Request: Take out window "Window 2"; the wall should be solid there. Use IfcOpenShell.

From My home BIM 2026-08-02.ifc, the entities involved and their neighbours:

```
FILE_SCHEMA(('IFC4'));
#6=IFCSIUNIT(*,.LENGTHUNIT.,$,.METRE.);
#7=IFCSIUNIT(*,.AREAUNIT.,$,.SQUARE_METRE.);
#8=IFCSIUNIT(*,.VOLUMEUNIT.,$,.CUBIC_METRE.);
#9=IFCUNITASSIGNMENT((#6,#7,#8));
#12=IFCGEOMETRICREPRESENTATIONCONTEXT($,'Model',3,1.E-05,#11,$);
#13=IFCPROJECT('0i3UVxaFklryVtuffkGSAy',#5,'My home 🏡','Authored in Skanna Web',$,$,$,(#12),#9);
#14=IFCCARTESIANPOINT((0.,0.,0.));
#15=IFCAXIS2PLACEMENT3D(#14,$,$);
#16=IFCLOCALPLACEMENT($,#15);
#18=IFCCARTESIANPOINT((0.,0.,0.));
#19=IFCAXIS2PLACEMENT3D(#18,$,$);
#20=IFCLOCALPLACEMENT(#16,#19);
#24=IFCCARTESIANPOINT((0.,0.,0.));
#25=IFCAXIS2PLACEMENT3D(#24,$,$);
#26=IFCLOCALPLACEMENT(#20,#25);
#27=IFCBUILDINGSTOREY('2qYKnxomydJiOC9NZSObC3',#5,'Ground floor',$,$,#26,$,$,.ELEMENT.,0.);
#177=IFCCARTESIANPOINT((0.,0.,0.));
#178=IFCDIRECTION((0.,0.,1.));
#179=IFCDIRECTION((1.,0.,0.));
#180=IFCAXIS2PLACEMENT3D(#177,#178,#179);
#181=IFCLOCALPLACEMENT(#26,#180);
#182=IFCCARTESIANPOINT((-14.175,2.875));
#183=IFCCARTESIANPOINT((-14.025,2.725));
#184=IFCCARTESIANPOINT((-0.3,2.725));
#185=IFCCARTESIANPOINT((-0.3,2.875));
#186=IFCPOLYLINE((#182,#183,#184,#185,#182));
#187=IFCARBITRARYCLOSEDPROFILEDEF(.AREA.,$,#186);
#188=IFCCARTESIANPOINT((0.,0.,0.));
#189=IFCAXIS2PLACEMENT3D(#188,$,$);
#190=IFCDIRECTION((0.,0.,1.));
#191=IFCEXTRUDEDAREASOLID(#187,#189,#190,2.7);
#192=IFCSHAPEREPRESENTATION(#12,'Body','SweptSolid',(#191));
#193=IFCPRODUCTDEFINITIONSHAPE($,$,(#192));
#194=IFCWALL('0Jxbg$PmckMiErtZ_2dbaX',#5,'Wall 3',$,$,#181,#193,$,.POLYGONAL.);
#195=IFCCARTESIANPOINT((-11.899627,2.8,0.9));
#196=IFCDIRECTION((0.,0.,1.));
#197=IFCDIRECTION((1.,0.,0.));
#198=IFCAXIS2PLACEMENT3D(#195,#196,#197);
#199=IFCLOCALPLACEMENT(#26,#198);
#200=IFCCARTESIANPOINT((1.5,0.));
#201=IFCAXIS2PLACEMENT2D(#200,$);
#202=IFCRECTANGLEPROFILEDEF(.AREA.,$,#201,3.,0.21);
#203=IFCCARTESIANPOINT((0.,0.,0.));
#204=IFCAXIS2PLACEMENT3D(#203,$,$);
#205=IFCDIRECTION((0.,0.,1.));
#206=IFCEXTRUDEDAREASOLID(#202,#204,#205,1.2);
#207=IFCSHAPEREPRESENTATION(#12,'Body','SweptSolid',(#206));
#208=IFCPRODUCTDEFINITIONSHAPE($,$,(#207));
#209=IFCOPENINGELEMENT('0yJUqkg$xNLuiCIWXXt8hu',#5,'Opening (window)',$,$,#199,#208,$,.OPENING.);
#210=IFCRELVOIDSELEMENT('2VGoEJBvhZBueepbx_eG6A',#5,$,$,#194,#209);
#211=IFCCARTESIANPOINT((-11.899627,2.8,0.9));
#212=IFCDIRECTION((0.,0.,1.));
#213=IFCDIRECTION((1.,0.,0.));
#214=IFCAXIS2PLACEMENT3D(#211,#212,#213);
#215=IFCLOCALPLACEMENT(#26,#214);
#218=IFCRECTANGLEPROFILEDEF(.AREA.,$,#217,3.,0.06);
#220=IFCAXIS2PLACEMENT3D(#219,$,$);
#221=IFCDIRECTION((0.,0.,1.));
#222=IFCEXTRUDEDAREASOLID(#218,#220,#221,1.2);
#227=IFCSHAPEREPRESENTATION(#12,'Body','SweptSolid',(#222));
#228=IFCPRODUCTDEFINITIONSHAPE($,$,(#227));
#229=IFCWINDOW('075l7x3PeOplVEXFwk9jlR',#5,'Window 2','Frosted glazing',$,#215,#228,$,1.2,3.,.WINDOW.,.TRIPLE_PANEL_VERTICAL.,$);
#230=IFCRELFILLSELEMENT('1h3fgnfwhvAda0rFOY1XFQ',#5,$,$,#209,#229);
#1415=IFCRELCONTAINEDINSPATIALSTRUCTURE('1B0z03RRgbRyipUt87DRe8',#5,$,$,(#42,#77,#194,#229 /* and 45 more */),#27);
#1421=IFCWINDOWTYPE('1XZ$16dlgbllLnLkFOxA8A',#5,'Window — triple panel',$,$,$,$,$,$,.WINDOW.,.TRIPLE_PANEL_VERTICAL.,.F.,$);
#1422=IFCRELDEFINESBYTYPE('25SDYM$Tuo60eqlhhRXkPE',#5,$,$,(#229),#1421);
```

```python
import ifcopenshell
import ifcopenshell.api.feature
import ifcopenshell.api.root
import ifcopenshell.geom
import ifcopenshell.util.shape

model = ifcopenshell.open("My home BIM 2026-08-02.ifc")
settings = ifcopenshell.geom.settings()


def volume(element):
    """Net volume in cubic metres, openings subtracted."""
    shape = ifcopenshell.geom.create_shape(settings, element)
    return ifcopenshell.util.shape.get_volume(shape.geometry)


window = model.by_guid("075l7x3PeOplVEXFwk9jlR")
opening = window.FillsVoids[0].RelatingOpeningElement
wall = opening.VoidsElements[0].RelatingBuildingElement
before = volume(wall)

ifcopenshell.api.root.remove_product(model, product=window)
ifcopenshell.api.feature.remove_feature(model, feature=opening)

after = volume(wall)

print(f"wall volume {before:.3f} -> {after:.3f} m3")

model.write("My home BIM 2026-08-02_rev.ifc")
```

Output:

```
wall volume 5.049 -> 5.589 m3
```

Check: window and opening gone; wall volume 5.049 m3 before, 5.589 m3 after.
